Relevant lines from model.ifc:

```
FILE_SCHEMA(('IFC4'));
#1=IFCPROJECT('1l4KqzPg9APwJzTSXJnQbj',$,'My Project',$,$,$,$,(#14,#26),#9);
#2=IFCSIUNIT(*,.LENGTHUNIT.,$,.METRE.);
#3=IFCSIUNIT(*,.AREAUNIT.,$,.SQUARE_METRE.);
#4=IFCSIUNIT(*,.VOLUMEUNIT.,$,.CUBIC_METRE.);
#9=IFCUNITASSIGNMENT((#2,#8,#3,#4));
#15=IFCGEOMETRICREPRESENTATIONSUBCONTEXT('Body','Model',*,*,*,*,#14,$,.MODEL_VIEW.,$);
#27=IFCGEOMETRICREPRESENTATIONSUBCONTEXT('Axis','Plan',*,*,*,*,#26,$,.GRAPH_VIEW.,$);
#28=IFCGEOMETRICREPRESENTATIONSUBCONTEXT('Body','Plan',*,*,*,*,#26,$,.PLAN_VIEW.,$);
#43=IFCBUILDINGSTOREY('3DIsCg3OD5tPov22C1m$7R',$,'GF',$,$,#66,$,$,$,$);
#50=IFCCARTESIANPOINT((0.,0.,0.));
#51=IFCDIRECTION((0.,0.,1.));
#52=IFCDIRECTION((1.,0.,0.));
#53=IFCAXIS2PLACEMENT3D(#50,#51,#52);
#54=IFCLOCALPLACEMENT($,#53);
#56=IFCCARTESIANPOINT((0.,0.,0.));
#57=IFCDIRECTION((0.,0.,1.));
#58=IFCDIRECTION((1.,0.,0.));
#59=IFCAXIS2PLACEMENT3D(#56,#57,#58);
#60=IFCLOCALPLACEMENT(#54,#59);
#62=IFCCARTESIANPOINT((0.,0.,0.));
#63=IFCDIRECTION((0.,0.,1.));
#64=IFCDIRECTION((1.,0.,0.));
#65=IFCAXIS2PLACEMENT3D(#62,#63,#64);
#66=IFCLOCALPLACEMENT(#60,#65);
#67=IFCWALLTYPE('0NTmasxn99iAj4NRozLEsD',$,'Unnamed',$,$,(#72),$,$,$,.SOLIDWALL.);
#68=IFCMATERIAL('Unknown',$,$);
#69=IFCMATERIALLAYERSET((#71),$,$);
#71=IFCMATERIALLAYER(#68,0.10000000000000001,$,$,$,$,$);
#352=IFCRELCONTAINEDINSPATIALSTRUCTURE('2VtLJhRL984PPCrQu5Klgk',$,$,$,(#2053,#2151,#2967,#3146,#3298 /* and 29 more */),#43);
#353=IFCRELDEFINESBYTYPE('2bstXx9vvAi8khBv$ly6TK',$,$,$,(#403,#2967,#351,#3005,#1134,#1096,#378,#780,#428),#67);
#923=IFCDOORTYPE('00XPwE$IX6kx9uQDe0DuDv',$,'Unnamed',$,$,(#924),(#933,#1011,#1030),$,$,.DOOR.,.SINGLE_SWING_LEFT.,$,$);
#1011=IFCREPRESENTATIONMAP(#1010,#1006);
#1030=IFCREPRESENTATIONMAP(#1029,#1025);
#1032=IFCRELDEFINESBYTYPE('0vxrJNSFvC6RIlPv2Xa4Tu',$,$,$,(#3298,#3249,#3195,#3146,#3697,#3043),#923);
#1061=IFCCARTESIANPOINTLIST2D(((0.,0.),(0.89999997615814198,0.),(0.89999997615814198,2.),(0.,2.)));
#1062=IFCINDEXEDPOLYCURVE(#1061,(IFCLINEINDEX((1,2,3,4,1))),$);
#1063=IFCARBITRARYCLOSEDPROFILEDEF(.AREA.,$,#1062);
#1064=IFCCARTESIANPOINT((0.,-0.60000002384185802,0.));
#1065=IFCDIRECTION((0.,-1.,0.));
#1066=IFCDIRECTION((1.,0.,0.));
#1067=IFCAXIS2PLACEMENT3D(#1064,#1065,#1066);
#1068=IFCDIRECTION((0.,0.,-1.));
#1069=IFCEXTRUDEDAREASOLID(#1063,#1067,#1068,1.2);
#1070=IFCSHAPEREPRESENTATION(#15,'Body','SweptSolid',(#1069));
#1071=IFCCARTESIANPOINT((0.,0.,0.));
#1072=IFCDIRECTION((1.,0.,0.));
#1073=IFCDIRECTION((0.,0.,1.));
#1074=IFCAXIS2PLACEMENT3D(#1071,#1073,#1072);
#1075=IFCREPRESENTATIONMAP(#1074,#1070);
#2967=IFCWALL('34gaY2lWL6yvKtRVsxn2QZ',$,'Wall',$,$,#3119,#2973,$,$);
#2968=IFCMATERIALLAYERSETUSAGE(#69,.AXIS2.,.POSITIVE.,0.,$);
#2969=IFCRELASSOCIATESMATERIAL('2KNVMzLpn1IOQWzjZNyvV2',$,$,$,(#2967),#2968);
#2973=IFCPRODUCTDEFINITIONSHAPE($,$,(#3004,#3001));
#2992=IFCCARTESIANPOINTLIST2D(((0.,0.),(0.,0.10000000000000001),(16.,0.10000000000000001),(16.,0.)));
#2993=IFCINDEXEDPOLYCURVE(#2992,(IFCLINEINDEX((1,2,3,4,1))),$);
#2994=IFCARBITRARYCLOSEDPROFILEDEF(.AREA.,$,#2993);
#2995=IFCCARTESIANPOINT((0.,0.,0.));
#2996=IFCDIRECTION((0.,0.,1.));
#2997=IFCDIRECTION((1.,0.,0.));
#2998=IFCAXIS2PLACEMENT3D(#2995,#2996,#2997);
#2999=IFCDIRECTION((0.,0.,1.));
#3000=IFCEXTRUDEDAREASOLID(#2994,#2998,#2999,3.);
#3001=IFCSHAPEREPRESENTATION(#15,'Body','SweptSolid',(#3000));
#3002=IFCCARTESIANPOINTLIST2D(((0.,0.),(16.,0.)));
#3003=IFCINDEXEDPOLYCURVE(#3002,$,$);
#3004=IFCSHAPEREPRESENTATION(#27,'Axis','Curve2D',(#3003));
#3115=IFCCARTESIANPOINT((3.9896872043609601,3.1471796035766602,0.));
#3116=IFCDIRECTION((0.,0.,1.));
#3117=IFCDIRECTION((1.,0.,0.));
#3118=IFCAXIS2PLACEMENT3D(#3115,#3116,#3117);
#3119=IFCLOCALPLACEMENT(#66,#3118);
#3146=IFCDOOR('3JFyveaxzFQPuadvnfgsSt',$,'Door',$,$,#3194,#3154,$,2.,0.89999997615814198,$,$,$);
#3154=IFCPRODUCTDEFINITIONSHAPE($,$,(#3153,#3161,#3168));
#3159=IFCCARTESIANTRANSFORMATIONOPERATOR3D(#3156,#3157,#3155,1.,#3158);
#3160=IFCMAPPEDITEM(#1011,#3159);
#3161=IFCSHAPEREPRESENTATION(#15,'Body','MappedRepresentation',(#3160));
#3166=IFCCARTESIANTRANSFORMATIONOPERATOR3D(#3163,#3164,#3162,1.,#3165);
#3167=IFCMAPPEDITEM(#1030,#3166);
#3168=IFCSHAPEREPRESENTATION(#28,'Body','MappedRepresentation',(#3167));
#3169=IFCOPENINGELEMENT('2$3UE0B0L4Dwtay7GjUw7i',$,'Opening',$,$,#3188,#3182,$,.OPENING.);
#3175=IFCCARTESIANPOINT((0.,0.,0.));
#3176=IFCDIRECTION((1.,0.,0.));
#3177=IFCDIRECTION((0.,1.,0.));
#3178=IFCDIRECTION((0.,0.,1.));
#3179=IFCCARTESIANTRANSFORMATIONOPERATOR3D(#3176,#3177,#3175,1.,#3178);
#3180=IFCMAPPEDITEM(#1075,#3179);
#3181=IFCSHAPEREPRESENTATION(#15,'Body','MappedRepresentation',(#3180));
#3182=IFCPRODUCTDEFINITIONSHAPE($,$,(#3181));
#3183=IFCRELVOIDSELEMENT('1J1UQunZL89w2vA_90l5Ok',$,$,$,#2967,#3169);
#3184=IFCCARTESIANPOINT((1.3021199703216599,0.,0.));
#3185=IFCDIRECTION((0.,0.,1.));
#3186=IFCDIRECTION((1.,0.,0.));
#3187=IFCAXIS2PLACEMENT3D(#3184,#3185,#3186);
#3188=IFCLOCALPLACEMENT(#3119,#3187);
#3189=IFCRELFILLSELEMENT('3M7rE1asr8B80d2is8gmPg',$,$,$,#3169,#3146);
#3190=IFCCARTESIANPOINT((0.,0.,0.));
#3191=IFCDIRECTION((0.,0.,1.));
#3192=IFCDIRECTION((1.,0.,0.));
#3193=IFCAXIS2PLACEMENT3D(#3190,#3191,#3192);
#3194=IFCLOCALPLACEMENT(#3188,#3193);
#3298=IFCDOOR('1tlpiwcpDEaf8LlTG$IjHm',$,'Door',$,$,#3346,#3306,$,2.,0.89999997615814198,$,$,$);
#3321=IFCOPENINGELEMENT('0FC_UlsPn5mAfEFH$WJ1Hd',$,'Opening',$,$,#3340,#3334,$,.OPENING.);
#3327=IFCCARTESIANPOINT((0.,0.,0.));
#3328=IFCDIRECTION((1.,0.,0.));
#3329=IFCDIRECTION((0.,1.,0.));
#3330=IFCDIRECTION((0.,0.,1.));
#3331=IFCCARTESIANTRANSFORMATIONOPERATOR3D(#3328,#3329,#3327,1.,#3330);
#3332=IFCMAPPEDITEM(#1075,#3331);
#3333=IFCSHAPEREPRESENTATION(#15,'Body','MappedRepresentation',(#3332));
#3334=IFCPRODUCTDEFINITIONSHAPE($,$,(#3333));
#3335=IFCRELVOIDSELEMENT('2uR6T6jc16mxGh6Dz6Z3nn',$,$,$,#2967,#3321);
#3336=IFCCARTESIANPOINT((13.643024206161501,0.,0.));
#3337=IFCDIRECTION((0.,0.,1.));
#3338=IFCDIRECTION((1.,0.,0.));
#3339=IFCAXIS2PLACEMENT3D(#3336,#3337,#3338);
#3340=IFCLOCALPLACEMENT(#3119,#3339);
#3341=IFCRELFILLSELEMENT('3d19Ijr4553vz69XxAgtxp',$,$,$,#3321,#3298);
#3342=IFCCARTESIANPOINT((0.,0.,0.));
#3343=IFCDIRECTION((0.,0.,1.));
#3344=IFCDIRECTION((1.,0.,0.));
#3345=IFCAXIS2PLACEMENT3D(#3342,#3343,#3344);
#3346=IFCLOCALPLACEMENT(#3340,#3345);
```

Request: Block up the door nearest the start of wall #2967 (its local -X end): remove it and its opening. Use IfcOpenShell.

```python
import ifcopenshell
import ifcopenshell.api.feature
import ifcopenshell.api.root
import ifcopenshell.geom
import ifcopenshell.util.shape

model = ifcopenshell.open("model.ifc")
settings = ifcopenshell.geom.settings()


def volume(element):
    """Net volume in cubic metres, openings subtracted."""
    shape = ifcopenshell.geom.create_shape(settings, element)
    return ifcopenshell.util.shape.get_volume(shape.geometry)


door = model.by_guid("3JFyveaxzFQPuadvnfgsSt")
opening = door.FillsVoids[0].RelatingOpeningElement
wall = opening.VoidsElements[0].RelatingBuildingElement
before = volume(wall)

ifcopenshell.api.root.remove_product(model, product=door)
ifcopenshell.api.feature.remove_feature(model, feature=opening)

after = volume(wall)

print(f"wall volume {before:.3f} -> {after:.3f} m3")

model.write("model_v2.ifc")
```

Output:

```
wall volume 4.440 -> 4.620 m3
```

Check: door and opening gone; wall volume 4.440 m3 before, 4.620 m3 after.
